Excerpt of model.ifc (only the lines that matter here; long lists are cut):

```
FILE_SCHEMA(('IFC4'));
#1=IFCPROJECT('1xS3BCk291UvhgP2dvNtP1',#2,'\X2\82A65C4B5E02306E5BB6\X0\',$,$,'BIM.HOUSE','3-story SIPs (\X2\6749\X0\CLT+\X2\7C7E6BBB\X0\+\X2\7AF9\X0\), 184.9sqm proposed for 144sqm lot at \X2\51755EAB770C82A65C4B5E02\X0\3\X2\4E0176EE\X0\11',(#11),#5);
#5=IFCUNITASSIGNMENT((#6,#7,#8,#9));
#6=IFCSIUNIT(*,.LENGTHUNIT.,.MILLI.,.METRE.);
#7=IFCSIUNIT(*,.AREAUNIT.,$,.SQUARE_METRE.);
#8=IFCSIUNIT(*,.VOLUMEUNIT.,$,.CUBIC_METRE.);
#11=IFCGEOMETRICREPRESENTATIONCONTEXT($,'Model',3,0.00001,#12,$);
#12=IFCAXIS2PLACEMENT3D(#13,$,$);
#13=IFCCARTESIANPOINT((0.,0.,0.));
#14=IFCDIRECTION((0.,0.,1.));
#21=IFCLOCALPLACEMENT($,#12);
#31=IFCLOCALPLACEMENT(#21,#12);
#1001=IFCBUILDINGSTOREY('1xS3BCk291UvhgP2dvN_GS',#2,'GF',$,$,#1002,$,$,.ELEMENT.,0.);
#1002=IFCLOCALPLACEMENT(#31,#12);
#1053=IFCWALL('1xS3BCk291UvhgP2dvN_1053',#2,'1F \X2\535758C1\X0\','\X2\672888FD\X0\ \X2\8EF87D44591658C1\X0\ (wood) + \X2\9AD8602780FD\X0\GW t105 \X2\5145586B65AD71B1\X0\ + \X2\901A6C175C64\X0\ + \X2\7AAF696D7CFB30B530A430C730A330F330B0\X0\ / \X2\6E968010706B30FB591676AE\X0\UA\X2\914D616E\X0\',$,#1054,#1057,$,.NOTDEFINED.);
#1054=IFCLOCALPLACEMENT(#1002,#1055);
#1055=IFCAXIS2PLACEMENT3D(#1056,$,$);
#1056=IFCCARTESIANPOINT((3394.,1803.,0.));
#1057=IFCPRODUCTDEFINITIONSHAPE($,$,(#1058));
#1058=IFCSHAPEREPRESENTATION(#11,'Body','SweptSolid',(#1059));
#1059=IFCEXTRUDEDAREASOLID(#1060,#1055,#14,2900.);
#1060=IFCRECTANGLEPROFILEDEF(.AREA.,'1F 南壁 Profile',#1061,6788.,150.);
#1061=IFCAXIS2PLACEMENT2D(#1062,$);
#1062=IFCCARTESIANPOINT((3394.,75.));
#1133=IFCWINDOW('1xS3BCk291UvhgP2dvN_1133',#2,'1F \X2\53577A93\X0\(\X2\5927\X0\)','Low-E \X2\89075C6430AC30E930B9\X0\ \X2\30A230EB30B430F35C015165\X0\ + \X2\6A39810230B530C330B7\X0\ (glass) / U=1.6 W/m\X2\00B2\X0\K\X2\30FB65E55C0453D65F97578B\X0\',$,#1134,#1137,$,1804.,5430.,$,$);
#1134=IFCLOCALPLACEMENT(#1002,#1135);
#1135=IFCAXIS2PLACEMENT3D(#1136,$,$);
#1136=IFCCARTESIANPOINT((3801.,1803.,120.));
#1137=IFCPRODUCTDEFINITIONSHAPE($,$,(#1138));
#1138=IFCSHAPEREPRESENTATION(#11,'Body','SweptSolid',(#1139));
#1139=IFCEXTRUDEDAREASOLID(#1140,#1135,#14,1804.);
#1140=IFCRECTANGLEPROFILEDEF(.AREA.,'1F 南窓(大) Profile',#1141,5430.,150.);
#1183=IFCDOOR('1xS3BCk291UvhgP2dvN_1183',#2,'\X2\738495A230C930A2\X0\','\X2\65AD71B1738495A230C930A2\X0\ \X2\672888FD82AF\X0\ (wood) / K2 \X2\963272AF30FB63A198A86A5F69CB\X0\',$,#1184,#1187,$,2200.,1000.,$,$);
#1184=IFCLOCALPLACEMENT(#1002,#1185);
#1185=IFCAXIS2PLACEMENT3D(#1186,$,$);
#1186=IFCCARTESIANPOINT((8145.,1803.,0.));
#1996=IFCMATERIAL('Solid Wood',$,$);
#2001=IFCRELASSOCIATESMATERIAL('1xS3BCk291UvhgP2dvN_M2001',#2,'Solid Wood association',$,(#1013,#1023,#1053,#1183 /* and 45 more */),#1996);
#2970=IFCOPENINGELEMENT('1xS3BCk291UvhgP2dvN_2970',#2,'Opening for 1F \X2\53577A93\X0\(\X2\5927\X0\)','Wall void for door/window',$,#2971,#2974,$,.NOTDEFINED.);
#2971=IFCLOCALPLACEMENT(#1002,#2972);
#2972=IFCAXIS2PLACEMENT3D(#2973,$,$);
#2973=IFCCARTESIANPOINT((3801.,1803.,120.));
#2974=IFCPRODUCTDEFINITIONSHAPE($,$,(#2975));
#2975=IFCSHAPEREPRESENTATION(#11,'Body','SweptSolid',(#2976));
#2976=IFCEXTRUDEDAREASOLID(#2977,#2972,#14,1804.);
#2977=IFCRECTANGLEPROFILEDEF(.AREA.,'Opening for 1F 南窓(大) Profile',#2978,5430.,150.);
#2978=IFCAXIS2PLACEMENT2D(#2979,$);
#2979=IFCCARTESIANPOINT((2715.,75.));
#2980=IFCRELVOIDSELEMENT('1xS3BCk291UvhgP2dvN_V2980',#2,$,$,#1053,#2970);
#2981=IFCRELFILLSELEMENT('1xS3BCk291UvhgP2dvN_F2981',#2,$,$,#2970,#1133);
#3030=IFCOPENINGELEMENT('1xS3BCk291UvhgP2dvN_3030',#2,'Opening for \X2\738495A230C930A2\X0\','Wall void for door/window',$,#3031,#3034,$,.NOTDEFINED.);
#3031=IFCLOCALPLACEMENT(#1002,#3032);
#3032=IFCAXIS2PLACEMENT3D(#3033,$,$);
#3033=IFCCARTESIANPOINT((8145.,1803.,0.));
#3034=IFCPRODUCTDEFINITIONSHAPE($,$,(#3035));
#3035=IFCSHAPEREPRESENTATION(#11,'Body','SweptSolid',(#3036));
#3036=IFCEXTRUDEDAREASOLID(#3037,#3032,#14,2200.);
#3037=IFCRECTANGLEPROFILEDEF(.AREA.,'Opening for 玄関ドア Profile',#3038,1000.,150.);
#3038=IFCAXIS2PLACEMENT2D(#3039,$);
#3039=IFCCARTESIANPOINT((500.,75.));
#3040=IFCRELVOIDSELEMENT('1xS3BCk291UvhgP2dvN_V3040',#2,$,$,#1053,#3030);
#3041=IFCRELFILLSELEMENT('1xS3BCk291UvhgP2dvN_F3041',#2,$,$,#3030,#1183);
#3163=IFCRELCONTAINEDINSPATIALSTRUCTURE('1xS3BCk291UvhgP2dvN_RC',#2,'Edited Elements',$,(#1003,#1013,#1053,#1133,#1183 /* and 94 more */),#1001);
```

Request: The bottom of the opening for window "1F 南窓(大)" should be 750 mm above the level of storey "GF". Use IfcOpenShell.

```python
import numpy as np
import ifcopenshell
import ifcopenshell.api.geometry
import ifcopenshell.geom
import ifcopenshell.util.element
import ifcopenshell.util.placement
import ifcopenshell.util.shape
import ifcopenshell.util.unit

model = ifcopenshell.open("model.ifc")
unit_scale = ifcopenshell.util.unit.calculate_unit_scale(model)

window = model.by_id(1133)
opening = window.FillsVoids[0].RelatingOpeningElement
storey = ifcopenshell.util.element.get_container(window, ifc_class="IfcBuildingStorey")
level = ifcopenshell.util.placement.get_local_placement(storey.ObjectPlacement)[2, 3]

# The opening's origin need not be at the sill, so measure its lowest point.
shape = ifcopenshell.geom.create_shape(ifcopenshell.geom.settings(), opening)
bottom = ifcopenshell.util.shape.get_shape_bottom_elevation(shape, shape.geometry) / unit_scale
dz = level + 0.75 / unit_scale - bottom

shift = np.array([0.0, 0.0, dz])
# The window is not placed relative to its opening, so move both.
for product in (opening, window):
    matrix = ifcopenshell.util.placement.get_local_placement(product.ObjectPlacement)
    matrix[:3, 3] += shift
    ifcopenshell.api.geometry.edit_object_placement(model, product=product, matrix=matrix, is_si=False)

print(f"moved by {dz * unit_scale:+.3f} m")

model.write("model_rev.ifc")
```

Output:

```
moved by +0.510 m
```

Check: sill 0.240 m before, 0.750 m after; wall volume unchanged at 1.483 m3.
